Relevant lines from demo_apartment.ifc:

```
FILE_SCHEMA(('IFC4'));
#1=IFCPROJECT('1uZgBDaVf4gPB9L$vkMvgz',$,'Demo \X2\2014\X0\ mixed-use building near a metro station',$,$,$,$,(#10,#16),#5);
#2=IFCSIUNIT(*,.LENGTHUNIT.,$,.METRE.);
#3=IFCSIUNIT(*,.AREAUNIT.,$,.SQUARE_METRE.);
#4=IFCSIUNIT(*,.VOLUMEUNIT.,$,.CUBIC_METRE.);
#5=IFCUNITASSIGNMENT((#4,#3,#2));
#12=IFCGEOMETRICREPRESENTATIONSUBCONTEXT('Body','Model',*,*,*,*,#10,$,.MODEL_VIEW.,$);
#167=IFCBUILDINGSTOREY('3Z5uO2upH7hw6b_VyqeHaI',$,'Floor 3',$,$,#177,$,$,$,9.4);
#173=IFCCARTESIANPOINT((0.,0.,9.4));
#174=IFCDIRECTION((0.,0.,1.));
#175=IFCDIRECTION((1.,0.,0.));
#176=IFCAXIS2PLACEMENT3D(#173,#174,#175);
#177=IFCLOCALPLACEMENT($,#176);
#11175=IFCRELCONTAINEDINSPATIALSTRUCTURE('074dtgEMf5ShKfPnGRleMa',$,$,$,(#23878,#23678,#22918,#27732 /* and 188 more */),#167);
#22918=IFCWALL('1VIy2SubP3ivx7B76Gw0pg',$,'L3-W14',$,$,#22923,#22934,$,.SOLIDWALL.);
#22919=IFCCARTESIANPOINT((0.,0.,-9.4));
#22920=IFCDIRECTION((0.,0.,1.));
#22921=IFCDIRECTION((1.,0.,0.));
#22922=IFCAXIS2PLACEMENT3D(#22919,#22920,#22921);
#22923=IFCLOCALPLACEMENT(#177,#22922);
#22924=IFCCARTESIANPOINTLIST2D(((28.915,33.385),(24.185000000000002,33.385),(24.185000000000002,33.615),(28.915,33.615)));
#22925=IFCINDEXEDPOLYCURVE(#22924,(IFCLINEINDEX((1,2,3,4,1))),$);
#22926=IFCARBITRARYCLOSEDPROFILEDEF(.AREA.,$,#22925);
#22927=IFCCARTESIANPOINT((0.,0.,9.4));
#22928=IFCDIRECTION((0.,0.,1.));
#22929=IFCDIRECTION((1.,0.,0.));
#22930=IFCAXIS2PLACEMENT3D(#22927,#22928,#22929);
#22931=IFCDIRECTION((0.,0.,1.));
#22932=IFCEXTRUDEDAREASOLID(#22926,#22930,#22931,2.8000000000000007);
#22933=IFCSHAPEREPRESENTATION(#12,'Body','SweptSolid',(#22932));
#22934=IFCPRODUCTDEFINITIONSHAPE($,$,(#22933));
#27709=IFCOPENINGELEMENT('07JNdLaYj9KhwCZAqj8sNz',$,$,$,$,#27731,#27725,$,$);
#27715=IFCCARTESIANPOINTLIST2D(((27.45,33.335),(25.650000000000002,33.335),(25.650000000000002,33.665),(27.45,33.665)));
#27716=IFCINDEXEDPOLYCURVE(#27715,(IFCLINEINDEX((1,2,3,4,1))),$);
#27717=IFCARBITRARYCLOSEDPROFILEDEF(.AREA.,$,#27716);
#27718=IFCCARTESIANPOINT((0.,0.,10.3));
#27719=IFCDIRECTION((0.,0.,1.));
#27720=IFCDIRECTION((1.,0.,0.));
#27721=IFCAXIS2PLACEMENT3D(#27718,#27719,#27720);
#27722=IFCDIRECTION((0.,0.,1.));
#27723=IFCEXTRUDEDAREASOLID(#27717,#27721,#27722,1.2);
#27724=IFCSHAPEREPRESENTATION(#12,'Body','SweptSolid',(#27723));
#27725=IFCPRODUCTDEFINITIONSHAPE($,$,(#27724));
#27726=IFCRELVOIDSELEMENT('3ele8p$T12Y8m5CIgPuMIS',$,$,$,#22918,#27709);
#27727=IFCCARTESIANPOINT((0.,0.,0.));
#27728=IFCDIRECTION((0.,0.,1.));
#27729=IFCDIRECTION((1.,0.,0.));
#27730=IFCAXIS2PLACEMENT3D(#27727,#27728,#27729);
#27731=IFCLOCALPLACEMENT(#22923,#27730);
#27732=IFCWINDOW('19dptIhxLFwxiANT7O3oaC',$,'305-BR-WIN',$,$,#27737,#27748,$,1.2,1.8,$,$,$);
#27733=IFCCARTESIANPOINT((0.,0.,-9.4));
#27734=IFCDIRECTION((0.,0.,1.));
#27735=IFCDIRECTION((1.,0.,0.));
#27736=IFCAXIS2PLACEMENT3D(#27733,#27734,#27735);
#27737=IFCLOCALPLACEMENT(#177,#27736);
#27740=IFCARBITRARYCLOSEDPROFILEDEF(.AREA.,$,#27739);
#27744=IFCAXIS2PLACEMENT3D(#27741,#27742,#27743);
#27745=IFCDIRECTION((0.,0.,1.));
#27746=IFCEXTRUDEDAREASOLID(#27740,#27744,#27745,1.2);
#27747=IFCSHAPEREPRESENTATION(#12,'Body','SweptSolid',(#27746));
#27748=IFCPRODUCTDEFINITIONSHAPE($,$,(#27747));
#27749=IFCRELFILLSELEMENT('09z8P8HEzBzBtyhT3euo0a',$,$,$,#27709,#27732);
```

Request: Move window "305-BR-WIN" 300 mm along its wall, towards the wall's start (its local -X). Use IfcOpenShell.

```python
import ifcopenshell
import ifcopenshell.api.geometry
import ifcopenshell.util.placement

model = ifcopenshell.open("demo_apartment.ifc")

window = model.by_guid("19dptIhxLFwxiANT7O3oaC")
opening = window.FillsVoids[0].RelatingOpeningElement
wall = opening.VoidsElements[0].RelatingBuildingElement

wall_matrix = ifcopenshell.util.placement.get_local_placement(wall.ObjectPlacement)
shift = wall_matrix[:3, 0] * -0.3
before = ifcopenshell.util.placement.get_local_placement(window.ObjectPlacement)[:3, 3].copy()

# The window is not placed relative to its opening, so move both.
for product in (opening, window):
    matrix = ifcopenshell.util.placement.get_local_placement(product.ObjectPlacement)
    matrix[:3, 3] += shift
    ifcopenshell.api.geometry.edit_object_placement(model, product=product, matrix=matrix, is_si=False)

after = ifcopenshell.util.placement.get_local_placement(window.ObjectPlacement)[:3, 3]
print("window moved by", (after - before).round(3) + 0.0)

model.write("demo_apartment_rev.ifc")
```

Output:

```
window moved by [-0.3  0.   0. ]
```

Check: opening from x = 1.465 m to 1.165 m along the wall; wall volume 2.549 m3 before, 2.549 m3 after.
